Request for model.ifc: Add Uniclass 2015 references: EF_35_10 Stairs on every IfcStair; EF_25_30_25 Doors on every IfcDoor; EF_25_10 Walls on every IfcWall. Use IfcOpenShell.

First a look at what the model holds.

```python
import ifcopenshell

model = ifcopenshell.open("model.ifc")
print(model.schema)
print("classifications:", [c.Name for c in model.by_type("IfcClassification")])
for ifc_class in ("IfcDoor", "IfcRoof", "IfcStair", "IfcWall", "IfcWindow"):
    print(ifc_class, len(model.by_type(ifc_class)))
```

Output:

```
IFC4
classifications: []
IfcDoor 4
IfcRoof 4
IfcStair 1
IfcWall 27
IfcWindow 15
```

```python
import ifcopenshell
import ifcopenshell.api.classification

model = ifcopenshell.open("model.ifc")

system = ifcopenshell.api.classification.add_classification(model, classification="Uniclass 2015")

codes = {
    "IfcStair": ("EF_35_10", "Stairs"),
    "IfcDoor": ("EF_25_30_25", "Doors"),
    "IfcWall": ("EF_25_10", "Walls"),
}
for ifc_class, (code, name) in codes.items():
    products = model.by_type(ifc_class)
    ifcopenshell.api.classification.add_reference(
        model, products=products, classification=system, identification=code, name=name
    )
    print(code, len(products))

model.write("model_rev.ifc")
```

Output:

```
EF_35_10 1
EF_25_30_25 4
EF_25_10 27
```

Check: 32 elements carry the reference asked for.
